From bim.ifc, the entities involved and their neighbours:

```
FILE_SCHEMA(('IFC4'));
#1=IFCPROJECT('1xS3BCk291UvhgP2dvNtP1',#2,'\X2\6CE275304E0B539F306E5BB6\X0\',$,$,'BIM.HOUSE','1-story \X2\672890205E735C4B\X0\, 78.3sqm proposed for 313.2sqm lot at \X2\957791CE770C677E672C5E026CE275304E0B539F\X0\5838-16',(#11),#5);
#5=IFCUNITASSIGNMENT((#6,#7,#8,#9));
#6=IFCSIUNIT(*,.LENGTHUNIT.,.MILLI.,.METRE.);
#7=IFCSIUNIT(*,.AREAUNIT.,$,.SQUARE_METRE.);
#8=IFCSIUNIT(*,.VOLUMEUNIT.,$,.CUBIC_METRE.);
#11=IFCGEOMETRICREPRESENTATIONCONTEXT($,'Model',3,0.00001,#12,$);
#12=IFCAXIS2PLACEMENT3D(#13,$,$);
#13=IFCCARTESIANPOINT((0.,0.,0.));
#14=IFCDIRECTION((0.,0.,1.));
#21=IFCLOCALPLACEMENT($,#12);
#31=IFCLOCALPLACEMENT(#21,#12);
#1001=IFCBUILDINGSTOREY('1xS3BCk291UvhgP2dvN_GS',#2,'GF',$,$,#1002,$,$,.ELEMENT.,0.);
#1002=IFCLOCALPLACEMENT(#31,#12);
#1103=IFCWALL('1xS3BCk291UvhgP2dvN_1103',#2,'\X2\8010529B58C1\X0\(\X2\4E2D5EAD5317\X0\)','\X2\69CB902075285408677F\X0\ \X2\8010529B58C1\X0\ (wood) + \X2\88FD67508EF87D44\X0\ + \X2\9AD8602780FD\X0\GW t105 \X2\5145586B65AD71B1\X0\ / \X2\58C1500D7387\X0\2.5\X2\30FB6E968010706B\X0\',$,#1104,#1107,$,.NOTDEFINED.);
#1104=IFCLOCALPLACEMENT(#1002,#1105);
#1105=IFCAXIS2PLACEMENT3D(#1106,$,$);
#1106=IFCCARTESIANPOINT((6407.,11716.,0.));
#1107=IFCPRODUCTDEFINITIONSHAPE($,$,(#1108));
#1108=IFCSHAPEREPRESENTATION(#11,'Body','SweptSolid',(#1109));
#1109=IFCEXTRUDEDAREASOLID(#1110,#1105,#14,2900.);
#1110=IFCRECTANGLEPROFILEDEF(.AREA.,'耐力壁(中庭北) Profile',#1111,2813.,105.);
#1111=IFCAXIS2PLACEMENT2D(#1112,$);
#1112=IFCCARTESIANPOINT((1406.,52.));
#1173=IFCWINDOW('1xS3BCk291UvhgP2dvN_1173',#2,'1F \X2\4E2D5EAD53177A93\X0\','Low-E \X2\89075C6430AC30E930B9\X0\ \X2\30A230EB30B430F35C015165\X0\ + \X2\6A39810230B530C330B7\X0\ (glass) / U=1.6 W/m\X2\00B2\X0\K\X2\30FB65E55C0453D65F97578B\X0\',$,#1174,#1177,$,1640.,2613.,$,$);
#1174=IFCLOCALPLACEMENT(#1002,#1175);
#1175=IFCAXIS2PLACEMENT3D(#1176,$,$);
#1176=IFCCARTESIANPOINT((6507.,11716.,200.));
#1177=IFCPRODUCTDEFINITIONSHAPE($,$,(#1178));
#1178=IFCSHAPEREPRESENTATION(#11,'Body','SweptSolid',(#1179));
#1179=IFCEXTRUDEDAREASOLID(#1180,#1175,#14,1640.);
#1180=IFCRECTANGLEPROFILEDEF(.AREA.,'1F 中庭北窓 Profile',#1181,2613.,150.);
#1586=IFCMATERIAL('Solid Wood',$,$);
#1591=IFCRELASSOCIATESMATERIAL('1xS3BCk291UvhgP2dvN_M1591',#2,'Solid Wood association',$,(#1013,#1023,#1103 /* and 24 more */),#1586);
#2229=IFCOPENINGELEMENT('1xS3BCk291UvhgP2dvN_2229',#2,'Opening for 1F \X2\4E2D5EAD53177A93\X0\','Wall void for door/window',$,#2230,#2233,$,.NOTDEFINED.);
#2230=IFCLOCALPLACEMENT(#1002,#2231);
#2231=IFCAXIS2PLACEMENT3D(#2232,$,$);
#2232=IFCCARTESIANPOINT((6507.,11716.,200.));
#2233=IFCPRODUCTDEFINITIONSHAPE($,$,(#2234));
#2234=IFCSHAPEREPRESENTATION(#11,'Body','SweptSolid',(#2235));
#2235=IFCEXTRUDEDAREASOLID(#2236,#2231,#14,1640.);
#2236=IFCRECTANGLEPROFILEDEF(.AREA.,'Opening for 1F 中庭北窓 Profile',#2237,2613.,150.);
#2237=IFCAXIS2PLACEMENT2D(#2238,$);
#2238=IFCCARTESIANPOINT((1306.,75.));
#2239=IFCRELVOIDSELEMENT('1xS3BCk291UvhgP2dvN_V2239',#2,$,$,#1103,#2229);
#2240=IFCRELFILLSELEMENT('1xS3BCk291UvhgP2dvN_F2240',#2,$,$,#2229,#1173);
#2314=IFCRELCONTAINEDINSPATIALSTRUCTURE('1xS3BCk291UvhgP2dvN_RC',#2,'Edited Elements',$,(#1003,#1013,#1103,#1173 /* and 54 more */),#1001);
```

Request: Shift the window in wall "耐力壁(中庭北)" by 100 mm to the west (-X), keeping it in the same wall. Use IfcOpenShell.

```python
import ifcopenshell
import ifcopenshell.api.geometry
import ifcopenshell.util.placement

model = ifcopenshell.open("bim.ifc")

window = model.by_id(1173)
opening = window.FillsVoids[0].RelatingOpeningElement
wall = opening.VoidsElements[0].RelatingBuildingElement

wall_matrix = ifcopenshell.util.placement.get_local_placement(wall.ObjectPlacement)
shift = wall_matrix[:3, 0] * -100.0
before = ifcopenshell.util.placement.get_local_placement(window.ObjectPlacement)[:3, 3].copy()

# The window is not placed relative to its opening, so move both.
for product in (opening, window):
    matrix = ifcopenshell.util.placement.get_local_placement(product.ObjectPlacement)
    matrix[:3, 3] += shift
    ifcopenshell.api.geometry.edit_object_placement(model, product=product, matrix=matrix, is_si=False)

after = ifcopenshell.util.placement.get_local_placement(window.ObjectPlacement)[:3, 3]
print("window moved by", (after - before).round(3) + 0.0)

model.write("bim-out.ifc")
```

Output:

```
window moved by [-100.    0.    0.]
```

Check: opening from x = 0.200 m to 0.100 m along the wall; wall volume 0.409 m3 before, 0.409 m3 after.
